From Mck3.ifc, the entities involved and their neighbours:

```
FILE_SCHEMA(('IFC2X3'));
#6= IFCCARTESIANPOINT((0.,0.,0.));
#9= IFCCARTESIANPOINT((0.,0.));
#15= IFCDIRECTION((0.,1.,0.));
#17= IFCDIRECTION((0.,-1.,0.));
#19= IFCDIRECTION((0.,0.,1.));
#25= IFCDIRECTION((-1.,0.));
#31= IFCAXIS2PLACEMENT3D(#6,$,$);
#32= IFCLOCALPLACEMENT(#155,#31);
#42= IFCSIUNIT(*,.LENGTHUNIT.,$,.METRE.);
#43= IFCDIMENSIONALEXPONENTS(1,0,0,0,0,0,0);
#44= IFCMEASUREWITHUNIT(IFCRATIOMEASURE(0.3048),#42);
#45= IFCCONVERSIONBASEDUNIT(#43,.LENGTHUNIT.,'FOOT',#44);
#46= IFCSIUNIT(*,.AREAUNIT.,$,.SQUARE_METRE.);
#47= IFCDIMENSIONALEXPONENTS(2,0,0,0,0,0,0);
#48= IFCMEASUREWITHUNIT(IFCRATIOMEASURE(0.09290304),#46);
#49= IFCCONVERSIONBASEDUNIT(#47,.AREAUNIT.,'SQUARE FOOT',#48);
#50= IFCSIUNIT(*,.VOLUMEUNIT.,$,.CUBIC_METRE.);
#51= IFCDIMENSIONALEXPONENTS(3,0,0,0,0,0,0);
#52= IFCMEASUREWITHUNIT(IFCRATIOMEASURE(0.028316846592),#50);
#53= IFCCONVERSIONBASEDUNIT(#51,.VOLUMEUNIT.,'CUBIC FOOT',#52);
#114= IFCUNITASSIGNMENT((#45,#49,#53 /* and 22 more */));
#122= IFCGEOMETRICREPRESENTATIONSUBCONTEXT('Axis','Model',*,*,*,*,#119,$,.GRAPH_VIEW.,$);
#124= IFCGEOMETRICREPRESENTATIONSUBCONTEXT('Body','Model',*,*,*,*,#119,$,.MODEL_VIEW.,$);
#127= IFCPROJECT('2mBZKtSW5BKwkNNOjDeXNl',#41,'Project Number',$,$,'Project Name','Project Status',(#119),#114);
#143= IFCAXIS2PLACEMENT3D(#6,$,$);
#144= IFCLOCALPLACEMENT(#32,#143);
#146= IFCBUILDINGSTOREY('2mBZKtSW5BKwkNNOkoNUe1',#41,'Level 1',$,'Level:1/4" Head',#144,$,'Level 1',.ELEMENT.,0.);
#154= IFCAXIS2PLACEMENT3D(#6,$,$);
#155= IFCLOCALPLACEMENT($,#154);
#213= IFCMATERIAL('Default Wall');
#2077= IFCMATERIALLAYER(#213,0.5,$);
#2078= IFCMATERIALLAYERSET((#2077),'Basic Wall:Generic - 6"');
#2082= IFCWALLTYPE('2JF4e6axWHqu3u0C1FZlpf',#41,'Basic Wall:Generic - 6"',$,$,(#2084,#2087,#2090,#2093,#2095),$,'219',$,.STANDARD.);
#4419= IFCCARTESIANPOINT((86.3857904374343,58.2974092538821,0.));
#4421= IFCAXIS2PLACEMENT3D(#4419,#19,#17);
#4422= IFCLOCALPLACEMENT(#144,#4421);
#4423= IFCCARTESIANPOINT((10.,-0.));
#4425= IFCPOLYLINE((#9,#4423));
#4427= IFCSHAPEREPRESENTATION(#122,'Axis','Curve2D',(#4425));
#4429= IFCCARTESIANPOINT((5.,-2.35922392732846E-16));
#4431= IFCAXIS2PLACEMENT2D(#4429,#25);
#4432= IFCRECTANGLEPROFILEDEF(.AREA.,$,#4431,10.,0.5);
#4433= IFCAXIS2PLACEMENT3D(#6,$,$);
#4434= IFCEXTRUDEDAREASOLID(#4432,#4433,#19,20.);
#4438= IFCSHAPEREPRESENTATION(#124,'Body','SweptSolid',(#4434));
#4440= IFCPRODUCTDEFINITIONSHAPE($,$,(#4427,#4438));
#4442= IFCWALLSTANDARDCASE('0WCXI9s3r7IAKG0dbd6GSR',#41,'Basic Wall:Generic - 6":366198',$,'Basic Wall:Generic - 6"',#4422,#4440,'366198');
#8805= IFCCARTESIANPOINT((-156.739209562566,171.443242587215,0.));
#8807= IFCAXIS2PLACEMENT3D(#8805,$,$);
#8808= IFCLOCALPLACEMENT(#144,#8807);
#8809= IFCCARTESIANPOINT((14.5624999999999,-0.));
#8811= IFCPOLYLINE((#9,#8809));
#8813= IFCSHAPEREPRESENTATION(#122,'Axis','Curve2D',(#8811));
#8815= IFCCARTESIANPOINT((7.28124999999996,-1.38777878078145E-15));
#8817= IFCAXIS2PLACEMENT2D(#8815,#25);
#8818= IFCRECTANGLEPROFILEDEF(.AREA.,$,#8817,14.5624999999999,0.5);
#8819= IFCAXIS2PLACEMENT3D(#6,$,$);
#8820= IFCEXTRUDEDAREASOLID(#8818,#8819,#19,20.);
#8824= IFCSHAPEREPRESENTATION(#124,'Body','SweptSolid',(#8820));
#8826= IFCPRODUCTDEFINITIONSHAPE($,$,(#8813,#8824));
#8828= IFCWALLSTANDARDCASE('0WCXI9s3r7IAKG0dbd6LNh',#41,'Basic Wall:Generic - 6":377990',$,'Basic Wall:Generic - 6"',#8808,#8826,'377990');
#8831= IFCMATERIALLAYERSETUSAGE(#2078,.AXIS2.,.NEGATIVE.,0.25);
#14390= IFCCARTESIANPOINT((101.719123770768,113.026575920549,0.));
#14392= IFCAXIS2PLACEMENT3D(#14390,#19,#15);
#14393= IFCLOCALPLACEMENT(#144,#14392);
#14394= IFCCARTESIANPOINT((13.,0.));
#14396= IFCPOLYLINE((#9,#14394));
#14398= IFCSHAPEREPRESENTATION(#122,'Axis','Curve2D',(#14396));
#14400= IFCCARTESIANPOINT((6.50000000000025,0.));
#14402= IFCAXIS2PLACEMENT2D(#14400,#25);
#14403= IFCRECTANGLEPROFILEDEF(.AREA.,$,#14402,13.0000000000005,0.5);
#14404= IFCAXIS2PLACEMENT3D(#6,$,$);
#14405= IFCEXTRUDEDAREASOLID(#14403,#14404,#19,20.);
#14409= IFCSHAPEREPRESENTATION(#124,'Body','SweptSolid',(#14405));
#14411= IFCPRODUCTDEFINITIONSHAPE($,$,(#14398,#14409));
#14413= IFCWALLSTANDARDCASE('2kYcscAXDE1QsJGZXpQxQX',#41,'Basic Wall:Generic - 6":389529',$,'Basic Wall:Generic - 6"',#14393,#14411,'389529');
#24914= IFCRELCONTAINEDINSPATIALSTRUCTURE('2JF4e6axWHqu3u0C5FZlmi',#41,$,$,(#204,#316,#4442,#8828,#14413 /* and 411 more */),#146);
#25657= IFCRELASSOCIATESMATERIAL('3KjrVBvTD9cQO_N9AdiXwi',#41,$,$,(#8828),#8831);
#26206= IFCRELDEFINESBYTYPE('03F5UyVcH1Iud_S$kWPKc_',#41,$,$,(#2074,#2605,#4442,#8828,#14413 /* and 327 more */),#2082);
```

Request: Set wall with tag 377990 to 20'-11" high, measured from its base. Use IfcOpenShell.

```python
import ifcopenshell
import ifcopenshell.geom
import ifcopenshell.util.representation
import ifcopenshell.util.shape
import ifcopenshell.util.unit

model = ifcopenshell.open("Mck3.ifc")
unit_scale = ifcopenshell.util.unit.calculate_unit_scale(model)
settings = ifcopenshell.geom.settings()


def volume(element):
    """Net volume in cubic metres, openings subtracted."""
    shape = ifcopenshell.geom.create_shape(settings, element)
    return ifcopenshell.util.shape.get_volume(shape.geometry)


wall = model.by_guid("0WCXI9s3r7IAKG0dbd6LNh")
before = volume(wall)

body = ifcopenshell.util.representation.get_representation(wall, "Model", "Body")
solid = body.Items[0]
old_height = solid.Depth
solid.Depth = 251 * 0.0254 / unit_scale
after = volume(wall)

print(f"height {old_height:g} -> {solid.Depth:g}, volume {before:.3f} -> {after:.3f} m3")

model.write("Mck3_updated.ifc")
```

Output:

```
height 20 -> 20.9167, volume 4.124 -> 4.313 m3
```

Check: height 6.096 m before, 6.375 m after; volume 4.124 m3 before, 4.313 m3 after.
